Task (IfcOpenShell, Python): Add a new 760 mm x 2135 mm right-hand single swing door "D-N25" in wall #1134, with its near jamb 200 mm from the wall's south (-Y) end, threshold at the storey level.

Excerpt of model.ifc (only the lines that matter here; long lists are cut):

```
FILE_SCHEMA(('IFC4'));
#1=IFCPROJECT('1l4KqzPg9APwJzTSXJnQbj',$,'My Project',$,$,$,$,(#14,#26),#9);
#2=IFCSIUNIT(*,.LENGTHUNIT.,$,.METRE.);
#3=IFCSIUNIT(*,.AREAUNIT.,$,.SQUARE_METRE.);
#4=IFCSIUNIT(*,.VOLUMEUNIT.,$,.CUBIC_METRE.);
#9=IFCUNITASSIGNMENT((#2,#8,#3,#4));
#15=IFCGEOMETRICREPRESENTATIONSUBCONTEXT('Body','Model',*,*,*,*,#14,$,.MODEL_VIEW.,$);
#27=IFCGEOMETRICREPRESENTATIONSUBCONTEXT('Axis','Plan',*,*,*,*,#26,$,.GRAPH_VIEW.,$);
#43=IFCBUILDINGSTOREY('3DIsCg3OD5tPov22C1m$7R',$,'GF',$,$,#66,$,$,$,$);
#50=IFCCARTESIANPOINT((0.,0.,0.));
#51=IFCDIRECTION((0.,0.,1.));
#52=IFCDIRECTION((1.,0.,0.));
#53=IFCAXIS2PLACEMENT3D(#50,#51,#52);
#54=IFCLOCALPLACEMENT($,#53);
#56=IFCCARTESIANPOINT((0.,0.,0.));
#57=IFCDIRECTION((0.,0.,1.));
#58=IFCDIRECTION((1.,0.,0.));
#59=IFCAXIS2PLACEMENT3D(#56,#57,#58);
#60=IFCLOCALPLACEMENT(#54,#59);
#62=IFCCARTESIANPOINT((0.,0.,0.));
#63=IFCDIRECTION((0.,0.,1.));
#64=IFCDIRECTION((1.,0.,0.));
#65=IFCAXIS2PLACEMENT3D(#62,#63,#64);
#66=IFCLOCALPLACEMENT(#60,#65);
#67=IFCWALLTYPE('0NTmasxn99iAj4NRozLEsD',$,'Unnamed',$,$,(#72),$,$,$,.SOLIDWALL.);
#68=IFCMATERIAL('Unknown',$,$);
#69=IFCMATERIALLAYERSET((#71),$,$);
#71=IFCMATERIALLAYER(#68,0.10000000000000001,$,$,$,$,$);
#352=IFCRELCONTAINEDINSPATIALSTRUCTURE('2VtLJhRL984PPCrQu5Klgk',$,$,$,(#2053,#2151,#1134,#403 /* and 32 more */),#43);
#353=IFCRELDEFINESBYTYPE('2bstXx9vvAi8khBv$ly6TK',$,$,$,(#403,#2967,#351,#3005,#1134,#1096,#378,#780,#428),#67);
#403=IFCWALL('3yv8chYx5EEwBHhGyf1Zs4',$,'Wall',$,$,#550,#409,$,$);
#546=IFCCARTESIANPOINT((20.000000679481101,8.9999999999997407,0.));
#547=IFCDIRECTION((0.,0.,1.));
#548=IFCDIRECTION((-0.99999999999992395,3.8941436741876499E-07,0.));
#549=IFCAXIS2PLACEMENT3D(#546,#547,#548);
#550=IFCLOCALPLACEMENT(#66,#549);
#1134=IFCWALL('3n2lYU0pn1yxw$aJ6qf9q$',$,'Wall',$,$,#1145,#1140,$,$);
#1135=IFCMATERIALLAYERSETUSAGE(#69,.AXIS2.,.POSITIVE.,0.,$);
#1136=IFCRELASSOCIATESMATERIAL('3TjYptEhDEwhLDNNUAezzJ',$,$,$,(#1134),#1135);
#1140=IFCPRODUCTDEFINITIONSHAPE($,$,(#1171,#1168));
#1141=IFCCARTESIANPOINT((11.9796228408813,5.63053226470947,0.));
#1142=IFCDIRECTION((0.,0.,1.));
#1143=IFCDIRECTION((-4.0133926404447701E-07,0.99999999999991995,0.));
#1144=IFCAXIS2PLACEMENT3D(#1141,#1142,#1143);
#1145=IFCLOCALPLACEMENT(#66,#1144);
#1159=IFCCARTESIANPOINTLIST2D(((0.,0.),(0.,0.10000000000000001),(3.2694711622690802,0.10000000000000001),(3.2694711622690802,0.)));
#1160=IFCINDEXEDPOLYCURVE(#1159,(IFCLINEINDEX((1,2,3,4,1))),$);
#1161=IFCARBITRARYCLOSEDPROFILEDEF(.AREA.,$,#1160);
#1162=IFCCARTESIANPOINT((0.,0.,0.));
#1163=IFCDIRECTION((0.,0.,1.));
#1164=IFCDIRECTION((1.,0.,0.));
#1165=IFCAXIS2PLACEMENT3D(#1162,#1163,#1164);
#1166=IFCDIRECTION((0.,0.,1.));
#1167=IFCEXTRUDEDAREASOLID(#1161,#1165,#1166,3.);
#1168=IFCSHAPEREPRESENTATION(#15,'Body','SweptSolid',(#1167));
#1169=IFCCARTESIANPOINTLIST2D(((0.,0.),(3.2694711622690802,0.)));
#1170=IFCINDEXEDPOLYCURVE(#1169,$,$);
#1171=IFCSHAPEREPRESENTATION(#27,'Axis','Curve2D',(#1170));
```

```python
import numpy as np
import ifcopenshell
import ifcopenshell.api.feature
import ifcopenshell.api.geometry
import ifcopenshell.api.root
import ifcopenshell.api.spatial
import ifcopenshell.geom
import ifcopenshell.util.element
import ifcopenshell.util.placement
import ifcopenshell.util.representation
import ifcopenshell.util.shape
import ifcopenshell.util.unit

model = ifcopenshell.open("model.ifc")
unit_scale = ifcopenshell.util.unit.calculate_unit_scale(model)
settings = ifcopenshell.geom.settings()


def volume(element):
    """Net volume in cubic metres, openings subtracted."""
    shape = ifcopenshell.geom.create_shape(settings, element)
    return ifcopenshell.util.shape.get_volume(shape.geometry)


wall = model.by_guid("3n2lYU0pn1yxw$aJ6qf9q$")
storey = ifcopenshell.util.element.get_container(wall, ifc_class="IfcBuildingStorey")
context = ifcopenshell.util.representation.get_context(model, "Model", "Body", "MODEL_VIEW")
before = volume(wall)

width, height, from_end, sill = 0.76, 2.135, 0.2, 0.0  # metres

# The wall runs along its own X axis, and the end named is its -X end.
wall_shape = ifcopenshell.geom.create_shape(settings, wall)
x, y, z = ifcopenshell.util.shape.get_vertices(wall_shape.geometry).T
start = x.min() + from_end
face, thickness = float(y.min()), float(y.max() - y.min())
wall_matrix = ifcopenshell.util.placement.get_local_placement(wall.ObjectPlacement)
level = ifcopenshell.util.placement.get_local_placement(storey.ObjectPlacement)[2, 3]


def in_wall(x, y):
    """Placement at x, y metres in the wall's axes, at sill height."""
    matrix = wall_matrix.copy()
    matrix[:, 3] = wall_matrix @ np.array([x / unit_scale, y / unit_scale, 0.0, 1.0])
    matrix[2, 3] = level + sill / unit_scale
    return matrix


# Opening: a box that overshoots both wall faces by 50 mm.
opening = ifcopenshell.api.root.create_entity(model, ifc_class="IfcOpeningElement", predefined_type="OPENING")
box = ifcopenshell.api.geometry.add_wall_representation(
    model, context=context, length=width, height=height, thickness=thickness + 0.1
)
ifcopenshell.api.geometry.assign_representation(model, product=opening, representation=box)
ifcopenshell.api.geometry.edit_object_placement(model, product=opening, matrix=in_wall(start, face - 0.05), is_si=False)
ifcopenshell.api.feature.add_feature(model, feature=opening, element=wall)

door = ifcopenshell.api.root.create_entity(model, ifc_class="IfcDoor", name="D-N25", predefined_type="DOOR")
door.OverallWidth, door.OverallHeight = width / unit_scale, height / unit_scale
door.OperationType = "SINGLE_SWING_RIGHT"
body = ifcopenshell.api.geometry.add_door_representation(
    model,
    context=context,
    overall_width=door.OverallWidth,
    overall_height=door.OverallHeight,
    operation_type="SINGLE_SWING_RIGHT",
    lining_properties={"LiningDepth": thickness / unit_scale, "ThresholdDepth": thickness / unit_scale},
)
ifcopenshell.api.geometry.assign_representation(model, product=door, representation=body)
ifcopenshell.api.spatial.assign_container(model, products=[door], relating_structure=storey)
ifcopenshell.api.feature.add_filling(model, opening=opening, element=door)

# The lining spans the wall, so the door starts at the wall face.
ifcopenshell.api.geometry.edit_object_placement(model, product=door, matrix=in_wall(start, face), is_si=False)

after = volume(wall)

print(f"wall volume {before:.3f} -> {after:.3f} m3")

model.write("model_rev.ifc")
```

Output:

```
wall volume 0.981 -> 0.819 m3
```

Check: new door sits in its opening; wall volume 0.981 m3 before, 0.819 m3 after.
